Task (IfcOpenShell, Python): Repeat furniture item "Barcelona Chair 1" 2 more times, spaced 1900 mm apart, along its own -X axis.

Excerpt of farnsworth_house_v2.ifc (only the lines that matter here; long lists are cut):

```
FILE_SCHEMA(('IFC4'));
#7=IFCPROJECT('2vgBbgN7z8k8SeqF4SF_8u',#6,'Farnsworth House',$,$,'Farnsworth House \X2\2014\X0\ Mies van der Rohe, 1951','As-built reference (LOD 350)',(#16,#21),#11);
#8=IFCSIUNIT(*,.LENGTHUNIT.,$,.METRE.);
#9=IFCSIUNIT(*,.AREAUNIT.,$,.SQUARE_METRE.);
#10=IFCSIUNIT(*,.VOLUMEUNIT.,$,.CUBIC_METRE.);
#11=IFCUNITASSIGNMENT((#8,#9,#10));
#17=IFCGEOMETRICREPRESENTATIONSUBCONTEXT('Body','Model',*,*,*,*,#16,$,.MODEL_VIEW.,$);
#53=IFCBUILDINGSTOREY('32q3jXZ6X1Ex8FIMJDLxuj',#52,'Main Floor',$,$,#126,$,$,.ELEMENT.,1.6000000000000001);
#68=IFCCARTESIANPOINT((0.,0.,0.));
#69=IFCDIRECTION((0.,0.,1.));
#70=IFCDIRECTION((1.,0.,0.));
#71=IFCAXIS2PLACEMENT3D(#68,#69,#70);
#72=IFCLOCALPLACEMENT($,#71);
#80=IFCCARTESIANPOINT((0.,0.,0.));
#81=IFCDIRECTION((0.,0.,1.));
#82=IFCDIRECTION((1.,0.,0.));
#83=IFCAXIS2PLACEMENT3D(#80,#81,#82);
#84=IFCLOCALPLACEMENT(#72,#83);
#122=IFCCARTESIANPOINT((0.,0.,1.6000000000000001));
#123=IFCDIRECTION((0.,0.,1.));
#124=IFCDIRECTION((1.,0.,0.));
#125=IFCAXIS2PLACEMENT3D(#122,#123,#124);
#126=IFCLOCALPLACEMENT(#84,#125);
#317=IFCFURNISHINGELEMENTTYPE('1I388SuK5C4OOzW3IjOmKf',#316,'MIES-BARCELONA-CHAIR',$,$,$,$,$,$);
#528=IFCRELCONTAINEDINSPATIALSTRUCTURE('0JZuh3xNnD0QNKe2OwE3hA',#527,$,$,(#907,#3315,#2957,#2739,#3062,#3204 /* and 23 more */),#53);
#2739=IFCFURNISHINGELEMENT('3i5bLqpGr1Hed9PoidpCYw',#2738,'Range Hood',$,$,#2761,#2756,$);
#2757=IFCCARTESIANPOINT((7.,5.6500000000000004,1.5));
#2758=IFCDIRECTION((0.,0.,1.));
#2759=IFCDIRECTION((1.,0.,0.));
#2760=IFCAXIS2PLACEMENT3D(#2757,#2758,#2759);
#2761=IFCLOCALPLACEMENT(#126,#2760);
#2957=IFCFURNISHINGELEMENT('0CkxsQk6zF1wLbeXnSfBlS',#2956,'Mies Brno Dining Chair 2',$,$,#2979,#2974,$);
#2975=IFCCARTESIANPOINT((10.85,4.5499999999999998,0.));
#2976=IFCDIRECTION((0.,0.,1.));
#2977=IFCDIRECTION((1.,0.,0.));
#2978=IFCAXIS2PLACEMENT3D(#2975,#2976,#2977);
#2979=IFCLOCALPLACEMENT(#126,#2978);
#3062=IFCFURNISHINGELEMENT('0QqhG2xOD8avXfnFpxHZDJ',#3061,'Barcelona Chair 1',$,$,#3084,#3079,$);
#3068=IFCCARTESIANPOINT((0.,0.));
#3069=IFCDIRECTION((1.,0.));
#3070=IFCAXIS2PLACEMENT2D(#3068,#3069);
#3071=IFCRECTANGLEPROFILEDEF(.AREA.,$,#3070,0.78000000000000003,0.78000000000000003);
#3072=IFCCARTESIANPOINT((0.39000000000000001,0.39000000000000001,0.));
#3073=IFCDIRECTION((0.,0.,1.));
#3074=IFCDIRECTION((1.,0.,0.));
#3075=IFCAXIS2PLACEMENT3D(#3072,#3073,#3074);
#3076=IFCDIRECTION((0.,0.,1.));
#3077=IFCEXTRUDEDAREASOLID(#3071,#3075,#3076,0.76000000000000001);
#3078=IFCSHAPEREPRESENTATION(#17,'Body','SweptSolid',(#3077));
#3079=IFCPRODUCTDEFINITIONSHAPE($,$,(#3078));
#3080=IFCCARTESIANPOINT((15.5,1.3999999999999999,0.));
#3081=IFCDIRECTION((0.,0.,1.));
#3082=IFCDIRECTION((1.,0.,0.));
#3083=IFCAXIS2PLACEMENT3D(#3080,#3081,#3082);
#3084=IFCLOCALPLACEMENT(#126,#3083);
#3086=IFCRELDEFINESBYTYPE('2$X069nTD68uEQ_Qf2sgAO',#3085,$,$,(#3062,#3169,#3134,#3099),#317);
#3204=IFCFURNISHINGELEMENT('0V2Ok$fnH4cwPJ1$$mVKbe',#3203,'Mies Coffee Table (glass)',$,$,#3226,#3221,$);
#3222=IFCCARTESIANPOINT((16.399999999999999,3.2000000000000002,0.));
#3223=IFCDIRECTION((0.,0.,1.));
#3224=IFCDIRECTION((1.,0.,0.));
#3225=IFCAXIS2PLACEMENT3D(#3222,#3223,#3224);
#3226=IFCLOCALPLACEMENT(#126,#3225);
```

```python
import ifcopenshell
import ifcopenshell.api.geometry
import ifcopenshell.api.root
import ifcopenshell.util.element
import ifcopenshell.util.placement

model = ifcopenshell.open("farnsworth_house_v2.ifc")


def reuse_history(source, copy):
    """copy_class also copies each property set's owner history, people and application; keep the originals."""
    for rel in copy.IsDefinedBy:
        if rel.is_a("IfcRelDefinesByProperties") and (history := rel.RelatingPropertyDefinition.OwnerHistory):
            rel.RelatingPropertyDefinition.OwnerHistory = source.OwnerHistory
            ifcopenshell.util.element.remove_deep2(model, history)


source = model.by_guid("0QqhG2xOD8avXfnFpxHZDJ")
base = ifcopenshell.util.placement.get_local_placement(source.ObjectPlacement)
step = -base[:3, 0] * 1.9

for i in range(1, 3):
    copy = ifcopenshell.api.root.copy_class(model, product=source)
    copy.Representation = ifcopenshell.util.element.copy_deep(
        model, source.Representation, exclude=["IfcGeometricRepresentationContext", "IfcRepresentationMap"]
    )
    reuse_history(source, copy)
    matrix = base.copy()
    matrix[:3, 3] += i * step
    print("added at", matrix[:3, 3].round(3) + 0.0)
    ifcopenshell.api.geometry.edit_object_placement(model, product=copy, matrix=matrix, is_si=False)

model.write("farnsworth_house_v2_edited.ifc")
```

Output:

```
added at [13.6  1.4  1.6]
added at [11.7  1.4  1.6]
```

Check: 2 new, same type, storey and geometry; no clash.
